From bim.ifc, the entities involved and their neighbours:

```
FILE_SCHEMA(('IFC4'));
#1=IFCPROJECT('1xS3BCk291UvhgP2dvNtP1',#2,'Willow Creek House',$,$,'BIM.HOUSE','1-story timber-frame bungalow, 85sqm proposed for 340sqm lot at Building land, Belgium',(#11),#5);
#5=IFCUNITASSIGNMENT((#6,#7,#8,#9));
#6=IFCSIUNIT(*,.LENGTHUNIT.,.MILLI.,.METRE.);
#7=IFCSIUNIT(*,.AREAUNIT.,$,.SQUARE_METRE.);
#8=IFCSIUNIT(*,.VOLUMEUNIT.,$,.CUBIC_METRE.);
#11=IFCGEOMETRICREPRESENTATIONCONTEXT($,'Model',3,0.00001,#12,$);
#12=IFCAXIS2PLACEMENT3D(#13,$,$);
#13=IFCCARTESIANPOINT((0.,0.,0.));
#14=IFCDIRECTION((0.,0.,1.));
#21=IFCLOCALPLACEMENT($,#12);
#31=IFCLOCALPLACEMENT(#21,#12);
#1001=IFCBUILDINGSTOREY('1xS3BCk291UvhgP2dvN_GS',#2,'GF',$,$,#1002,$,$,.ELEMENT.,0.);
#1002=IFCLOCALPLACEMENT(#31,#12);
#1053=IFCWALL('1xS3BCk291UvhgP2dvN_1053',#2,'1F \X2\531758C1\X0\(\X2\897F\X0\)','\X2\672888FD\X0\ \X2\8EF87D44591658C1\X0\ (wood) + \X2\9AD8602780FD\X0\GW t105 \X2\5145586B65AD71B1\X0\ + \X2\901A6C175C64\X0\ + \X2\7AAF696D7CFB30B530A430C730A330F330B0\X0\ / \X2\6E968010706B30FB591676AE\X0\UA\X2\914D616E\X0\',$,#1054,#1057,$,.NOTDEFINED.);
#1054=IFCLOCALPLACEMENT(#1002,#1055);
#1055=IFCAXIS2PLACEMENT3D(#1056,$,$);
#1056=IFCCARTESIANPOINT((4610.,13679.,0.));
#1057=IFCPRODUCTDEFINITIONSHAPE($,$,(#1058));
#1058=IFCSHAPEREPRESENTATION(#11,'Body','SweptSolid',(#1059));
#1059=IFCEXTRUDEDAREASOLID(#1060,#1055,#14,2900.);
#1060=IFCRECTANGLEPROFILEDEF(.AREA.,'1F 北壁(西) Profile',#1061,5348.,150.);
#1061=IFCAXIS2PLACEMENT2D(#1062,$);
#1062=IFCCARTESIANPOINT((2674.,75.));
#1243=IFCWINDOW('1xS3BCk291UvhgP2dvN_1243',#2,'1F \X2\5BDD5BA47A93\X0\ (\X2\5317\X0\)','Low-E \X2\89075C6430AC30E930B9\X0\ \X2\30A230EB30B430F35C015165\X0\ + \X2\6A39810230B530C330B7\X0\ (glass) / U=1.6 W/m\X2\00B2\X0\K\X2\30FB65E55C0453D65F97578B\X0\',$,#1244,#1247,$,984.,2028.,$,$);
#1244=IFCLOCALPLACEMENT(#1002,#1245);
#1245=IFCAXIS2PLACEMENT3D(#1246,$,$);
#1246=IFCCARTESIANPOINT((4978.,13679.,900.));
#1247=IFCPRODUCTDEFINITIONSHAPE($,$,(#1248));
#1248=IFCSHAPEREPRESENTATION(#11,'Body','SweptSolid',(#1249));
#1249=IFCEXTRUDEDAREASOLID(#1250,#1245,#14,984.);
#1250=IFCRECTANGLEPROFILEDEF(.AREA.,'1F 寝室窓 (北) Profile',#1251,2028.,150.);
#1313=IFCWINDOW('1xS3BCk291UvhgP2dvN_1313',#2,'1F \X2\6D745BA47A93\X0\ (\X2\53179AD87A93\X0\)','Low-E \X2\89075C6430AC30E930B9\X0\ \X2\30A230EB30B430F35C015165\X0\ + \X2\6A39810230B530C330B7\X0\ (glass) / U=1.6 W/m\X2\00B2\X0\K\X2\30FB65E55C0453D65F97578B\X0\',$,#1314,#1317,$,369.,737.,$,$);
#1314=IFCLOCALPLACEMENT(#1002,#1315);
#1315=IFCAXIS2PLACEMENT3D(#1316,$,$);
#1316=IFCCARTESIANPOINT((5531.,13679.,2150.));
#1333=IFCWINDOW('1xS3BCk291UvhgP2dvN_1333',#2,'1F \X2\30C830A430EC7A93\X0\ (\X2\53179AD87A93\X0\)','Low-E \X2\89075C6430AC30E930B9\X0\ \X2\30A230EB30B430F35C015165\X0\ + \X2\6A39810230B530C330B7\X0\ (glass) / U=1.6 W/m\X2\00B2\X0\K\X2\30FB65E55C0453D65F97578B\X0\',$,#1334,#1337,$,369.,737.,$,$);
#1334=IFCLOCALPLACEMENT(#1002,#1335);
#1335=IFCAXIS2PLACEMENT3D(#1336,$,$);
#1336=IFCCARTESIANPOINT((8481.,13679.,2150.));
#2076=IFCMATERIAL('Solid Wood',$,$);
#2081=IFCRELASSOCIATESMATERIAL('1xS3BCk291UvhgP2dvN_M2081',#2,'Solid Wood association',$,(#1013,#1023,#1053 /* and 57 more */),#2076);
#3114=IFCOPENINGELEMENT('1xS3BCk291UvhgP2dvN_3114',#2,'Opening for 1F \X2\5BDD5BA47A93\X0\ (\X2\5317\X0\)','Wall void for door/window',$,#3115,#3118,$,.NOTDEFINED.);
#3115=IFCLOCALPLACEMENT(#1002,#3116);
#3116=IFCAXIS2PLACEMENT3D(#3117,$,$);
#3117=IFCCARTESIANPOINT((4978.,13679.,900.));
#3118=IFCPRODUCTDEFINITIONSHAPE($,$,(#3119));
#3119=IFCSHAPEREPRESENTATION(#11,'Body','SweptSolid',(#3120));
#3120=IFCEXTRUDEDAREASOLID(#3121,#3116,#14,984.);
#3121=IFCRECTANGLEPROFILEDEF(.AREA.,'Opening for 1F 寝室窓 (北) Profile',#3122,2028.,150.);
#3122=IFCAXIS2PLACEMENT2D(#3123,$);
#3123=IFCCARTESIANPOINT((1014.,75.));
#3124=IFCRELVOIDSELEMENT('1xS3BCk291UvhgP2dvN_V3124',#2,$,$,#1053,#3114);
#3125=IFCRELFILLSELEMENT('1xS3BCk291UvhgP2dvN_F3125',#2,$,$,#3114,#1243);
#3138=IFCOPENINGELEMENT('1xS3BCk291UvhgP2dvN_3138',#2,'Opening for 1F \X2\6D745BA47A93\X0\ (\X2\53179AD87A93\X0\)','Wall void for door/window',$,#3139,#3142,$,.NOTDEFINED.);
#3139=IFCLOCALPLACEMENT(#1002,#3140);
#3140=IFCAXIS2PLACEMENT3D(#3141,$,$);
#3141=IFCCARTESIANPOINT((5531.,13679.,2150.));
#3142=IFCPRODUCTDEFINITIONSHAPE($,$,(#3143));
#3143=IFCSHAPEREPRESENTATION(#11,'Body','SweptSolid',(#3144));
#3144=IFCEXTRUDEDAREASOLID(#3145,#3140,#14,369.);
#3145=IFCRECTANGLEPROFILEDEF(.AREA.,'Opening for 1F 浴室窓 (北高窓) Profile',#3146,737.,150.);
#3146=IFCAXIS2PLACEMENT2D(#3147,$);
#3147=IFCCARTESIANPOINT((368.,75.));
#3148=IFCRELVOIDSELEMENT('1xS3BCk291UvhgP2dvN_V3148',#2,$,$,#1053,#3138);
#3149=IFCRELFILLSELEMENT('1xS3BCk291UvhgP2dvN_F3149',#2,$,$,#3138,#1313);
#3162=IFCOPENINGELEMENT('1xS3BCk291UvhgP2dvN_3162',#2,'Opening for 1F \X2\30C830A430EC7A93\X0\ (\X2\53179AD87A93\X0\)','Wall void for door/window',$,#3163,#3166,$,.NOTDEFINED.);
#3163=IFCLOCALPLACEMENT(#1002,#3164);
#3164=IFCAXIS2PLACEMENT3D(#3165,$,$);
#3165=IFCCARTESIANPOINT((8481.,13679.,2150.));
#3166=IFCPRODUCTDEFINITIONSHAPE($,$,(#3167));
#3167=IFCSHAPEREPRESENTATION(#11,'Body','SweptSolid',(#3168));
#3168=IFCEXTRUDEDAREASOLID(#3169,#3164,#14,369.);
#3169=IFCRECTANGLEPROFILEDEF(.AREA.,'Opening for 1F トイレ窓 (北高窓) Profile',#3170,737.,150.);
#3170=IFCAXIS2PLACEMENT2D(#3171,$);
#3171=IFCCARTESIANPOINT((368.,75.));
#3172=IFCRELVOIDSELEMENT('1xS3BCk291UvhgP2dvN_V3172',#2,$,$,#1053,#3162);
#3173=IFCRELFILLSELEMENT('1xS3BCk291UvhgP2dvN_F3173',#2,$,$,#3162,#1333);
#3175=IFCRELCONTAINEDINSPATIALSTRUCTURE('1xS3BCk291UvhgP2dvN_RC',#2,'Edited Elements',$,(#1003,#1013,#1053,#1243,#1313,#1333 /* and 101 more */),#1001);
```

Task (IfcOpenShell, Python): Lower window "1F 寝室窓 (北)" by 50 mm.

```python
import numpy as np
import ifcopenshell
import ifcopenshell.api.geometry
import ifcopenshell.util.placement
import ifcopenshell.util.unit

model = ifcopenshell.open("bim.ifc")
unit_scale = ifcopenshell.util.unit.calculate_unit_scale(model)

window = model.by_guid("1xS3BCk291UvhgP2dvN_1243")
opening = window.FillsVoids[0].RelatingOpeningElement
dz = -50.0

shift = np.array([0.0, 0.0, dz])
# The window is not placed relative to its opening, so move both.
for product in (opening, window):
    matrix = ifcopenshell.util.placement.get_local_placement(product.ObjectPlacement)
    matrix[:3, 3] += shift
    ifcopenshell.api.geometry.edit_object_placement(model, product=product, matrix=matrix, is_si=False)

print(f"moved by {dz * unit_scale:+.3f} m")

model.write("bim_edited.ifc")
```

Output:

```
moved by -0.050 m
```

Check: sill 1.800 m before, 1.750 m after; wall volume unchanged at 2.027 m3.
